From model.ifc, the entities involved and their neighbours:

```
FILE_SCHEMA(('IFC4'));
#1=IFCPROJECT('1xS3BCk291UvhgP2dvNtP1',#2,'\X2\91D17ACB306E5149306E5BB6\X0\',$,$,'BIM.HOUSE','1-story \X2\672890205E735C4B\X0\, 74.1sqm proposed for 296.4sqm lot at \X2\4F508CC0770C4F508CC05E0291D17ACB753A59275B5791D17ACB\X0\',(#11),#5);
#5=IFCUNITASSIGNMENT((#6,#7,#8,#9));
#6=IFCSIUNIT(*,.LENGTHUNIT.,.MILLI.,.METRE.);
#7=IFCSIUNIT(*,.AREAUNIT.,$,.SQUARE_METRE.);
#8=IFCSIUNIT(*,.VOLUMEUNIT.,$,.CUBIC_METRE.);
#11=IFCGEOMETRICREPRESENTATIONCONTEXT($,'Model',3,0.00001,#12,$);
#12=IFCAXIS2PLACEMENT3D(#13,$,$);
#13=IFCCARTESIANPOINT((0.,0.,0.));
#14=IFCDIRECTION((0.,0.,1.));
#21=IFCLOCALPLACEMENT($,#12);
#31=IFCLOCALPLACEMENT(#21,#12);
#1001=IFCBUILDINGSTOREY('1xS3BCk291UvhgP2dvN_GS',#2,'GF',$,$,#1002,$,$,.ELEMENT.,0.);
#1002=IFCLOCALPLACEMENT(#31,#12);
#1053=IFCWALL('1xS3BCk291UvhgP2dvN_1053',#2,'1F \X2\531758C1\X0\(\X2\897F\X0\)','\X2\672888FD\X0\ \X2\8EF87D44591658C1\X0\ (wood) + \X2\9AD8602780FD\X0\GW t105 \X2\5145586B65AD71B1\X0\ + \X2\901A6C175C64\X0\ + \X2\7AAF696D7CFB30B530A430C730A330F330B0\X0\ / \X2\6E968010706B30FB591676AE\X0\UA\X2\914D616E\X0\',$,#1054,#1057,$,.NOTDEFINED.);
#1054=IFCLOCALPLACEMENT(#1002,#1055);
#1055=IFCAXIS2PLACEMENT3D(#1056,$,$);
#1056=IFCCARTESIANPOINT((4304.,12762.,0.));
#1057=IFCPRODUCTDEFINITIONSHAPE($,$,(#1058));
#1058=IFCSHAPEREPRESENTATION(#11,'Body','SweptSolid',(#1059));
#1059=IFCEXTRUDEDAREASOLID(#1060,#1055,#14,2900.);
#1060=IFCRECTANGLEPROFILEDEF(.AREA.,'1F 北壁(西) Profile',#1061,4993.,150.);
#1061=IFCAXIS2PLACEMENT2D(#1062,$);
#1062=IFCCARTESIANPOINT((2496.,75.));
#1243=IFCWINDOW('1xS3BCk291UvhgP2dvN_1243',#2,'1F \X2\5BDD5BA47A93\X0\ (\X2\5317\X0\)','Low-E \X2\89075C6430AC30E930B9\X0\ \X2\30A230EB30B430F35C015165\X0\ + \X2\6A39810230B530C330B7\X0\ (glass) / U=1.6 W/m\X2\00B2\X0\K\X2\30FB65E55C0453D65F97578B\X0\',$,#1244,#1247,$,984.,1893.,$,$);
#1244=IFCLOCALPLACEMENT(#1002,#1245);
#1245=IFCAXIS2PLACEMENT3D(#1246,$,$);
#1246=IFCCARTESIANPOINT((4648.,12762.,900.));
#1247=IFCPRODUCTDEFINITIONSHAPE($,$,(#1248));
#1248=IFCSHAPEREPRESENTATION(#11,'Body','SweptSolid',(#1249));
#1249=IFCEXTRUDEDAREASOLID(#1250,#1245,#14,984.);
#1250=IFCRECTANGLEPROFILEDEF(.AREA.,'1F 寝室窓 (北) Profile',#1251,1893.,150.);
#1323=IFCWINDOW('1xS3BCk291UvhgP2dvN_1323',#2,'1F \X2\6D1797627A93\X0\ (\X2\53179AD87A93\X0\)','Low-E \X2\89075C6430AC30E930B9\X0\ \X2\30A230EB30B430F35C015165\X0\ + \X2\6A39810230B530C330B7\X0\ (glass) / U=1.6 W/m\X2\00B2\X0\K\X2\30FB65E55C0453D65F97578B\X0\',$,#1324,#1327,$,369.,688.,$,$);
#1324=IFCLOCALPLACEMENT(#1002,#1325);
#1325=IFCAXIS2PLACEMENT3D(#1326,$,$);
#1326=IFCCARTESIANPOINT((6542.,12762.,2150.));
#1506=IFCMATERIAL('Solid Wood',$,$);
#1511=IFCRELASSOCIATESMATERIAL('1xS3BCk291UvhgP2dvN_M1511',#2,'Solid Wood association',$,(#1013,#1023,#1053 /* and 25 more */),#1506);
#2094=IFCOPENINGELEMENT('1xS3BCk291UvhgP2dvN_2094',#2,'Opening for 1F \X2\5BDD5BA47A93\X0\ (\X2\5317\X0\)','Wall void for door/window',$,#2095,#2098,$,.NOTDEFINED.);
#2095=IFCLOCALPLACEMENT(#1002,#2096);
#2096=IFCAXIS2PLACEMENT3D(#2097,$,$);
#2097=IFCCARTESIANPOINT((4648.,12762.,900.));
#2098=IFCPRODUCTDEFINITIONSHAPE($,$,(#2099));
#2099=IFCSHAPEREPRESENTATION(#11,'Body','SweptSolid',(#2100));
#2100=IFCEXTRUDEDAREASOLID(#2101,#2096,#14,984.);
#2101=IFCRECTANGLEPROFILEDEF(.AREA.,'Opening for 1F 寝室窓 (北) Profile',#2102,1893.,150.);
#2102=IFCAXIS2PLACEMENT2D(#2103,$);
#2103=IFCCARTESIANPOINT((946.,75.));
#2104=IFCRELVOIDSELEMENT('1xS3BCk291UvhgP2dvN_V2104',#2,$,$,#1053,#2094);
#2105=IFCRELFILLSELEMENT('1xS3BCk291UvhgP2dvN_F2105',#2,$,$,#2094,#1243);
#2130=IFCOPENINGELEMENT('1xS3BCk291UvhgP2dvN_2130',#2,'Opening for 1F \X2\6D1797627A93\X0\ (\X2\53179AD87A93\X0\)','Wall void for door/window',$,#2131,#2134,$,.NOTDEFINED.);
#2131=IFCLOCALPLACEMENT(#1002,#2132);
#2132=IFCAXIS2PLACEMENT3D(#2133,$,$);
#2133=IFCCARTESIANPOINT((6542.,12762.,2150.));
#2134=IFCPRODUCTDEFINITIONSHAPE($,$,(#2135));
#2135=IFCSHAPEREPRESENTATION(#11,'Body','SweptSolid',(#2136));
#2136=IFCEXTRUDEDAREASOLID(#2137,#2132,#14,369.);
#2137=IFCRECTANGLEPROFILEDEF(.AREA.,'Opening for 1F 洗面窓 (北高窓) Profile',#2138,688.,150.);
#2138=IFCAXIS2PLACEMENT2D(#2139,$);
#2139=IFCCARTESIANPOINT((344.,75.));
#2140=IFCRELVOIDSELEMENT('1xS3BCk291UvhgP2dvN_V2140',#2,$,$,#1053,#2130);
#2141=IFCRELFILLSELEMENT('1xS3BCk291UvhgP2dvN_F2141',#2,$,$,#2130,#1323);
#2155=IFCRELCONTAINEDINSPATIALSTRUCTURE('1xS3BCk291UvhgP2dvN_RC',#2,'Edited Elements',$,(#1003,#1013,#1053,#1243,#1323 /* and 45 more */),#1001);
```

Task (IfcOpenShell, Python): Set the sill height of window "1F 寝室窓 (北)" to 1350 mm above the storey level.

```python
import numpy as np
import ifcopenshell
import ifcopenshell.api.geometry
import ifcopenshell.geom
import ifcopenshell.util.element
import ifcopenshell.util.placement
import ifcopenshell.util.shape
import ifcopenshell.util.unit

model = ifcopenshell.open("model.ifc")
unit_scale = ifcopenshell.util.unit.calculate_unit_scale(model)

window = model.by_guid("1xS3BCk291UvhgP2dvN_1243")
opening = window.FillsVoids[0].RelatingOpeningElement
storey = ifcopenshell.util.element.get_container(window, ifc_class="IfcBuildingStorey")
level = ifcopenshell.util.placement.get_local_placement(storey.ObjectPlacement)[2, 3]

# The opening's origin need not be at the sill, so measure its lowest point.
shape = ifcopenshell.geom.create_shape(ifcopenshell.geom.settings(), opening)
bottom = ifcopenshell.util.shape.get_shape_bottom_elevation(shape, shape.geometry) / unit_scale
dz = level + 1.35 / unit_scale - bottom

shift = np.array([0.0, 0.0, dz])
# The window is not placed relative to its opening, so move both.
for product in (opening, window):
    matrix = ifcopenshell.util.placement.get_local_placement(product.ObjectPlacement)
    matrix[:3, 3] += shift
    ifcopenshell.api.geometry.edit_object_placement(model, product=product, matrix=matrix, is_si=False)

print(f"moved by {dz * unit_scale:+.3f} m")

model.write("model_edited.ifc")
```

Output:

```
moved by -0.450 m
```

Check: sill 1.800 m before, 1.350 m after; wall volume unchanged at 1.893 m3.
